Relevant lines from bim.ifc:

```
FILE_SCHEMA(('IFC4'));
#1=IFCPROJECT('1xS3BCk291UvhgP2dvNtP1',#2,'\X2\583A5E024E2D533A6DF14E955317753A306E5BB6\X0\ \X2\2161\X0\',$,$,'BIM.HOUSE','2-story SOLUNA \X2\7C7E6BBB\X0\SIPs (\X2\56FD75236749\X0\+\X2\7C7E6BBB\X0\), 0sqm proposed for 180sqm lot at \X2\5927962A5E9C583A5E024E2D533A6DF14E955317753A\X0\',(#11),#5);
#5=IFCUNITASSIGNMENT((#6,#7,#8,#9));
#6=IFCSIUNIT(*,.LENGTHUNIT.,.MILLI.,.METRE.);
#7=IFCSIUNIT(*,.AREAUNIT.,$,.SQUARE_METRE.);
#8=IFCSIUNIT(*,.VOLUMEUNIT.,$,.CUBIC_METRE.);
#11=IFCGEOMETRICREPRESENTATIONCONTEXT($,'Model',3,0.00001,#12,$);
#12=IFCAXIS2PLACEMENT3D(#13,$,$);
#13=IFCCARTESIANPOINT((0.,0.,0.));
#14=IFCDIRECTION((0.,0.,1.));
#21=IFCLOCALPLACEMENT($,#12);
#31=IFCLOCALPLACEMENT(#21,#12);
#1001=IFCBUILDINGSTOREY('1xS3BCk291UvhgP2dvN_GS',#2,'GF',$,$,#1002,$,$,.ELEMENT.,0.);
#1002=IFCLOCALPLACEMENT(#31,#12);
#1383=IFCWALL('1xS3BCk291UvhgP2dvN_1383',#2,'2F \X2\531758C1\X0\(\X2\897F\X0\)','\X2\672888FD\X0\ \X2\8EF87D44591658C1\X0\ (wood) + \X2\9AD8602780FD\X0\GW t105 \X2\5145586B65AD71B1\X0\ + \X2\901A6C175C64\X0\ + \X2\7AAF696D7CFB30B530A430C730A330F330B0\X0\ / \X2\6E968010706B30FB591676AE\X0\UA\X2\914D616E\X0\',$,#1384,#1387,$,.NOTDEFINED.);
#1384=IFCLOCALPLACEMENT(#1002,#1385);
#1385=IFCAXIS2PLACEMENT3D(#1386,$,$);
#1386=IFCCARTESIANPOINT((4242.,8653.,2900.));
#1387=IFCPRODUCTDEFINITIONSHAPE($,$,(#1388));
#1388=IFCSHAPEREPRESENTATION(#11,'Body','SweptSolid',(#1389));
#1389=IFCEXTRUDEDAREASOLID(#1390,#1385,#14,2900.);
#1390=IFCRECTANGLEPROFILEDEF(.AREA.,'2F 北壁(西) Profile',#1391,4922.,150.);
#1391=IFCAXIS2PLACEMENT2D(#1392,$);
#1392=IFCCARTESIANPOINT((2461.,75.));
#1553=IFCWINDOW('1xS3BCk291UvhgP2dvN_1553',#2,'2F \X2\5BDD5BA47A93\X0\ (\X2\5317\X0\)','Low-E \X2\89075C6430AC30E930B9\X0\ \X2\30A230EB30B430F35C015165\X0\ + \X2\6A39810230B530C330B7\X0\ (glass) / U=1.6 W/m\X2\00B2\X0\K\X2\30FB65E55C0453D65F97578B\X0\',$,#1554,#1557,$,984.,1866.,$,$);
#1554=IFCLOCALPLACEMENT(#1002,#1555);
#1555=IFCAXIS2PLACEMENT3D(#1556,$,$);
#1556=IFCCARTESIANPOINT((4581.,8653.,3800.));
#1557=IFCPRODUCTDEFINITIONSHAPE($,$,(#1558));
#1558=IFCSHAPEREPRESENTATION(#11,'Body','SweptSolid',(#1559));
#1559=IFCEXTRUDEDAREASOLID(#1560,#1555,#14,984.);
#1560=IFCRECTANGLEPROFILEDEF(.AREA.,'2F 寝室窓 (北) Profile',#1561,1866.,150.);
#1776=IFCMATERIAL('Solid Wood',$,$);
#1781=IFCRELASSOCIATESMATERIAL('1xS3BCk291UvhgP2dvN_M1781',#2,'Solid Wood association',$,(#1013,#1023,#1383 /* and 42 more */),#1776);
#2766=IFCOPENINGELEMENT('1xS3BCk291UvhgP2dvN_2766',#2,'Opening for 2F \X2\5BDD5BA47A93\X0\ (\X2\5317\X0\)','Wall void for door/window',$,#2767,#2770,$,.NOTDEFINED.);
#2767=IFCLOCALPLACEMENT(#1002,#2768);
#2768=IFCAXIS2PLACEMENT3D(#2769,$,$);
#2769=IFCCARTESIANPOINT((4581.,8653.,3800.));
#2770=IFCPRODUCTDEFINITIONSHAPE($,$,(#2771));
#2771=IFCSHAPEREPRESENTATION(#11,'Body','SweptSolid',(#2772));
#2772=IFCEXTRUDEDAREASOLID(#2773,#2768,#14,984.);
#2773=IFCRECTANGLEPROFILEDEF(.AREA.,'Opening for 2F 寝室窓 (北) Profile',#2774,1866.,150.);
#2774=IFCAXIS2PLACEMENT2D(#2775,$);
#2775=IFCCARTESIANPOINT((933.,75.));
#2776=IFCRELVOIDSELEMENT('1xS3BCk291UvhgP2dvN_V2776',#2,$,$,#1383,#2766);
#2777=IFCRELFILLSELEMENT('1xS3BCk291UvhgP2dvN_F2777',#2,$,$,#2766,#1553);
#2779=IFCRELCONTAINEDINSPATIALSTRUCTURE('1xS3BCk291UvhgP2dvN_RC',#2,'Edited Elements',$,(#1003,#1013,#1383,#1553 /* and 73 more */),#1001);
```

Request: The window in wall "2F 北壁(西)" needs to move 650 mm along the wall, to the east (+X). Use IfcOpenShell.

```python
import ifcopenshell
import ifcopenshell.api.geometry
import ifcopenshell.util.placement

model = ifcopenshell.open("bim.ifc")

window = model.by_guid("1xS3BCk291UvhgP2dvN_1553")
opening = window.FillsVoids[0].RelatingOpeningElement
wall = opening.VoidsElements[0].RelatingBuildingElement

wall_matrix = ifcopenshell.util.placement.get_local_placement(wall.ObjectPlacement)
shift = wall_matrix[:3, 0] * 650.0
before = ifcopenshell.util.placement.get_local_placement(window.ObjectPlacement)[:3, 3].copy()

# The window is not placed relative to its opening, so move both.
for product in (opening, window):
    matrix = ifcopenshell.util.placement.get_local_placement(product.ObjectPlacement)
    matrix[:3, 3] += shift
    ifcopenshell.api.geometry.edit_object_placement(model, product=product, matrix=matrix, is_si=False)

after = ifcopenshell.util.placement.get_local_placement(window.ObjectPlacement)[:3, 3]
print("window moved by", (after - before).round(3) + 0.0)

model.write("bim_edited.ifc")
```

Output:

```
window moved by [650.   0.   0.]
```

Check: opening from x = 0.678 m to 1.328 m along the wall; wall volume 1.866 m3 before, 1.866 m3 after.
